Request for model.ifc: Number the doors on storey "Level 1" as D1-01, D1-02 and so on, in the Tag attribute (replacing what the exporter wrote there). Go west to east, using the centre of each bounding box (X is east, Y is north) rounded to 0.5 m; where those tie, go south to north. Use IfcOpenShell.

First a look at what the model holds.

```python
import ifcopenshell
import ifcopenshell.util.element
import ifcopenshell.util.placement

model = ifcopenshell.open("model.ifc")
print(model.schema)
storey = next(s for s in model.by_type("IfcBuildingStorey") if s.Name == "Level 1")
doors = [e for e in ifcopenshell.util.element.get_decomposition(storey) if e.is_a("IfcDoor")]
for e in sorted(doors, key=lambda e: e.id()):
    origin = ifcopenshell.util.placement.get_local_placement(e.ObjectPlacement)[:3, 3]
    print(e.id(), e.Tag, e.Name, origin.round(2) + 0.0, sep=" | ")
```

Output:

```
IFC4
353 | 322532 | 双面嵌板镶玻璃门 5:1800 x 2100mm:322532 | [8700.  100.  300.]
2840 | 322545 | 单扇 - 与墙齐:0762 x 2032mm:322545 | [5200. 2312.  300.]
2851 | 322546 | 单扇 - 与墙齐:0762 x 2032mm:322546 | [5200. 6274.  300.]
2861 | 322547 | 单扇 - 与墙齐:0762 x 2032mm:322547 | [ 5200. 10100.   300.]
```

```python
import ifcopenshell
import ifcopenshell.geom
import ifcopenshell.util.element
import ifcopenshell.util.shape

model = ifcopenshell.open("model.ifc")
settings = ifcopenshell.geom.settings()
settings.set("use-world-coords", True)


def centre(element):
    shape = ifcopenshell.geom.create_shape(settings, element)
    return ifcopenshell.util.shape.get_bbox_centroid(shape.geometry)


storey = next(s for s in model.by_type("IfcBuildingStorey") if s.Name == "Level 1")
doors = [e for e in ifcopenshell.util.element.get_decomposition(storey) if e.is_a("IfcDoor")]

# Insertion points can sit at a corner or the storey origin, so sort by the geometry (in metres).
centres = {e: centre(e) for e in doors}
doors.sort(key=lambda e: (round(centres[e][0] / 0.5), centres[e][1]))

for i, e in enumerate(doors, start=1):
    number = f"D1-{i:02d}"
    e.Tag = number
    print(e.id(), number)

model.write("model-out.ifc")
```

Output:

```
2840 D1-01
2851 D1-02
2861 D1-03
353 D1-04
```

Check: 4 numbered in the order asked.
